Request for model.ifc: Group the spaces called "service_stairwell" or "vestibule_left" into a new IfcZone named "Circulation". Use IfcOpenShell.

First a look at what the model holds.

```python
import ifcopenshell

model = ifcopenshell.open("model.ifc")
print(model.schema)
seen = {}
for space in model.by_type("IfcSpace"):
    seen[space.LongName] = seen.get(space.LongName, 0) + 1
for name, count in sorted(seen.items(), key=str):
    print(count, "x", name)
print("zones:", [z.Name for z in model.by_type("IfcZone")][:20])
```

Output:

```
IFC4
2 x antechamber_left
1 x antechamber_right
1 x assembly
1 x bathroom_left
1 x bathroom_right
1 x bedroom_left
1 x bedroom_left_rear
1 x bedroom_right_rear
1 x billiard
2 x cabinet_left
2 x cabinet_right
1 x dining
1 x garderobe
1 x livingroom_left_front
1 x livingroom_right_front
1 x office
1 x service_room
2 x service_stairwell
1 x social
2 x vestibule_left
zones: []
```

```python
import ifcopenshell
import ifcopenshell.api.group
import ifcopenshell.api.root

model = ifcopenshell.open("model.ifc")

names = {"service_stairwell", "vestibule_left"}
spaces = [s for s in model.by_type("IfcSpace") if s.LongName in names]

zone = ifcopenshell.api.root.create_entity(model, ifc_class="IfcZone", name="Circulation")
ifcopenshell.api.group.assign_group(model, products=spaces, group=zone)
print(len(spaces), "spaces in", zone.Name)

model.write("model-out.ifc")
```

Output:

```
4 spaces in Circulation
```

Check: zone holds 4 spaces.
